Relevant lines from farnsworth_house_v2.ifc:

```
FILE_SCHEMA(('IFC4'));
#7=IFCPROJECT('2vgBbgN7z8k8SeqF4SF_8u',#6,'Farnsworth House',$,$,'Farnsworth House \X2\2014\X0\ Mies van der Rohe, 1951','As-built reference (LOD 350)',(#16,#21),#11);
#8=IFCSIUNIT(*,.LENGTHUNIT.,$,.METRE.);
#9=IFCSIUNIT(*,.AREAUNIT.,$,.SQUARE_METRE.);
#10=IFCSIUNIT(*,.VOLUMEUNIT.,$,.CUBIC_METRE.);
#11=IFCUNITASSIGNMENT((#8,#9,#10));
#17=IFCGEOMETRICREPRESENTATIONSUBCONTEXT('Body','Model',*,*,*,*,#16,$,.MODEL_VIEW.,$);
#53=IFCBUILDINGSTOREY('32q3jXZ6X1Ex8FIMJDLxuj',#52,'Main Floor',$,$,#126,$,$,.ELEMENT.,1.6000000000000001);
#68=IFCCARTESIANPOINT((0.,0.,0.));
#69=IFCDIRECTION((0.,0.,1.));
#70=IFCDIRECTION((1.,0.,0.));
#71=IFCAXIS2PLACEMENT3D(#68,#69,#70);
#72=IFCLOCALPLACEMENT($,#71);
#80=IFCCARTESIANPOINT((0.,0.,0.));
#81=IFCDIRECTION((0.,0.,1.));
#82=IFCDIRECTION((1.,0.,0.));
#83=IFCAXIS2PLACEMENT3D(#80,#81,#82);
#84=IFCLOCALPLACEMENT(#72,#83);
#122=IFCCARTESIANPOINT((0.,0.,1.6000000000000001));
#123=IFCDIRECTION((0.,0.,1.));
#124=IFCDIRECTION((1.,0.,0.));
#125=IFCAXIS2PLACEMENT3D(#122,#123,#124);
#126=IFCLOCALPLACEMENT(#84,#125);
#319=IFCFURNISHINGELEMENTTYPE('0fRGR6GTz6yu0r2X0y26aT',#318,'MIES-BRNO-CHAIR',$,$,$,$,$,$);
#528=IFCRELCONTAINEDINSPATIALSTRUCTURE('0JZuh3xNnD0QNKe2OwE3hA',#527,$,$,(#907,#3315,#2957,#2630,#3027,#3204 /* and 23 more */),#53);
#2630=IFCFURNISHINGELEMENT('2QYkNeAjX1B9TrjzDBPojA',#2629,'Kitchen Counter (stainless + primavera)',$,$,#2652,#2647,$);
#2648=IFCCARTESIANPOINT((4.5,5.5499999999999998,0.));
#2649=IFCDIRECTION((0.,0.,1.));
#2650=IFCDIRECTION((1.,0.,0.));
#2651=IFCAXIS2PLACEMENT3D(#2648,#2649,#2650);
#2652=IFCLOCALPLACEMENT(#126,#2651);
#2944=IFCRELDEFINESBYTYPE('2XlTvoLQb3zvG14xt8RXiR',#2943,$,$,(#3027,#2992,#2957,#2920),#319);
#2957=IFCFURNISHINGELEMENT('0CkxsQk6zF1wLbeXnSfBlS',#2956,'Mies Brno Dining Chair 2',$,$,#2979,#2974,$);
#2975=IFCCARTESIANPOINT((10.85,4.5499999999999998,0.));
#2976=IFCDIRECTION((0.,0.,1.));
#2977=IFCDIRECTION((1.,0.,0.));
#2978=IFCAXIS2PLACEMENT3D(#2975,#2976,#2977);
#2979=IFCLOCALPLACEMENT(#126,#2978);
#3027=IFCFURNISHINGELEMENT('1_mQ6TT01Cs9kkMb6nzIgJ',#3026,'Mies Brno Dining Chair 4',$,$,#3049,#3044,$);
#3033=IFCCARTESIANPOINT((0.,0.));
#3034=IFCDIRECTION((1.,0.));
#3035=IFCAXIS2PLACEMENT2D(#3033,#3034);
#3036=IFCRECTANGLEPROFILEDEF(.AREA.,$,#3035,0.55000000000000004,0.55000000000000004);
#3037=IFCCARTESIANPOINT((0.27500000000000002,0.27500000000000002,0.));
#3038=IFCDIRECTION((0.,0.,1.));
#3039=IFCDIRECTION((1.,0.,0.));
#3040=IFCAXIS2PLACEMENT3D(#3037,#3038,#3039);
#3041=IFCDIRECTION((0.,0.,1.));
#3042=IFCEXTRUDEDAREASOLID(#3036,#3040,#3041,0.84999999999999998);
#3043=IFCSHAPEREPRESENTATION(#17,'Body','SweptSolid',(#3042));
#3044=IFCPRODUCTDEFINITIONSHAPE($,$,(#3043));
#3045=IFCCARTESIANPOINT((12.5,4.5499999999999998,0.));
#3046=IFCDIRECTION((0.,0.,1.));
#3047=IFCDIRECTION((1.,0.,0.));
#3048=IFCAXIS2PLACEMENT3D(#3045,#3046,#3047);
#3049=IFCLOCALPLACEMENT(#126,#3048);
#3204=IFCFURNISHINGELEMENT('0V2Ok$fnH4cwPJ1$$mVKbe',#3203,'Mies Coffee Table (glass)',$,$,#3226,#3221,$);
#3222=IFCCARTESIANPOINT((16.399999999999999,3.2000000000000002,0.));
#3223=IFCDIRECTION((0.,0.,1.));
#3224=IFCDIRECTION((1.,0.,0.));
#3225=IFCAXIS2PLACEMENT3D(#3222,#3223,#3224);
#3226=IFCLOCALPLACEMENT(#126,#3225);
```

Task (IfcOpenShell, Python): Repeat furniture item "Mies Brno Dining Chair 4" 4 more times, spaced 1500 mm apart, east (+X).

```python
import numpy as np
import ifcopenshell
import ifcopenshell.api.geometry
import ifcopenshell.api.root
import ifcopenshell.util.element
import ifcopenshell.util.placement

model = ifcopenshell.open("farnsworth_house_v2.ifc")


def reuse_history(source, copy):
    """copy_class also copies each property set's owner history, people and application; keep the originals."""
    for rel in copy.IsDefinedBy:
        if rel.is_a("IfcRelDefinesByProperties") and (history := rel.RelatingPropertyDefinition.OwnerHistory):
            rel.RelatingPropertyDefinition.OwnerHistory = source.OwnerHistory
            ifcopenshell.util.element.remove_deep2(model, history)


source = model.by_id(3027)
base = ifcopenshell.util.placement.get_local_placement(source.ObjectPlacement)
step = np.array([1.0, 0.0, 0.0]) * 1.5

for i in range(1, 5):
    copy = ifcopenshell.api.root.copy_class(model, product=source)
    copy.Representation = ifcopenshell.util.element.copy_deep(
        model, source.Representation, exclude=["IfcGeometricRepresentationContext", "IfcRepresentationMap"]
    )
    reuse_history(source, copy)
    matrix = base.copy()
    matrix[:3, 3] += i * step
    print("added at", matrix[:3, 3].round(3) + 0.0)
    ifcopenshell.api.geometry.edit_object_placement(model, product=copy, matrix=matrix, is_si=False)

model.write("farnsworth_house_v2_edited.ifc")
```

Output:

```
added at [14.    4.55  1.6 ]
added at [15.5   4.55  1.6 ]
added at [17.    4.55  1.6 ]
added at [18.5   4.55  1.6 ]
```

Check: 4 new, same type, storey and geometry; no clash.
